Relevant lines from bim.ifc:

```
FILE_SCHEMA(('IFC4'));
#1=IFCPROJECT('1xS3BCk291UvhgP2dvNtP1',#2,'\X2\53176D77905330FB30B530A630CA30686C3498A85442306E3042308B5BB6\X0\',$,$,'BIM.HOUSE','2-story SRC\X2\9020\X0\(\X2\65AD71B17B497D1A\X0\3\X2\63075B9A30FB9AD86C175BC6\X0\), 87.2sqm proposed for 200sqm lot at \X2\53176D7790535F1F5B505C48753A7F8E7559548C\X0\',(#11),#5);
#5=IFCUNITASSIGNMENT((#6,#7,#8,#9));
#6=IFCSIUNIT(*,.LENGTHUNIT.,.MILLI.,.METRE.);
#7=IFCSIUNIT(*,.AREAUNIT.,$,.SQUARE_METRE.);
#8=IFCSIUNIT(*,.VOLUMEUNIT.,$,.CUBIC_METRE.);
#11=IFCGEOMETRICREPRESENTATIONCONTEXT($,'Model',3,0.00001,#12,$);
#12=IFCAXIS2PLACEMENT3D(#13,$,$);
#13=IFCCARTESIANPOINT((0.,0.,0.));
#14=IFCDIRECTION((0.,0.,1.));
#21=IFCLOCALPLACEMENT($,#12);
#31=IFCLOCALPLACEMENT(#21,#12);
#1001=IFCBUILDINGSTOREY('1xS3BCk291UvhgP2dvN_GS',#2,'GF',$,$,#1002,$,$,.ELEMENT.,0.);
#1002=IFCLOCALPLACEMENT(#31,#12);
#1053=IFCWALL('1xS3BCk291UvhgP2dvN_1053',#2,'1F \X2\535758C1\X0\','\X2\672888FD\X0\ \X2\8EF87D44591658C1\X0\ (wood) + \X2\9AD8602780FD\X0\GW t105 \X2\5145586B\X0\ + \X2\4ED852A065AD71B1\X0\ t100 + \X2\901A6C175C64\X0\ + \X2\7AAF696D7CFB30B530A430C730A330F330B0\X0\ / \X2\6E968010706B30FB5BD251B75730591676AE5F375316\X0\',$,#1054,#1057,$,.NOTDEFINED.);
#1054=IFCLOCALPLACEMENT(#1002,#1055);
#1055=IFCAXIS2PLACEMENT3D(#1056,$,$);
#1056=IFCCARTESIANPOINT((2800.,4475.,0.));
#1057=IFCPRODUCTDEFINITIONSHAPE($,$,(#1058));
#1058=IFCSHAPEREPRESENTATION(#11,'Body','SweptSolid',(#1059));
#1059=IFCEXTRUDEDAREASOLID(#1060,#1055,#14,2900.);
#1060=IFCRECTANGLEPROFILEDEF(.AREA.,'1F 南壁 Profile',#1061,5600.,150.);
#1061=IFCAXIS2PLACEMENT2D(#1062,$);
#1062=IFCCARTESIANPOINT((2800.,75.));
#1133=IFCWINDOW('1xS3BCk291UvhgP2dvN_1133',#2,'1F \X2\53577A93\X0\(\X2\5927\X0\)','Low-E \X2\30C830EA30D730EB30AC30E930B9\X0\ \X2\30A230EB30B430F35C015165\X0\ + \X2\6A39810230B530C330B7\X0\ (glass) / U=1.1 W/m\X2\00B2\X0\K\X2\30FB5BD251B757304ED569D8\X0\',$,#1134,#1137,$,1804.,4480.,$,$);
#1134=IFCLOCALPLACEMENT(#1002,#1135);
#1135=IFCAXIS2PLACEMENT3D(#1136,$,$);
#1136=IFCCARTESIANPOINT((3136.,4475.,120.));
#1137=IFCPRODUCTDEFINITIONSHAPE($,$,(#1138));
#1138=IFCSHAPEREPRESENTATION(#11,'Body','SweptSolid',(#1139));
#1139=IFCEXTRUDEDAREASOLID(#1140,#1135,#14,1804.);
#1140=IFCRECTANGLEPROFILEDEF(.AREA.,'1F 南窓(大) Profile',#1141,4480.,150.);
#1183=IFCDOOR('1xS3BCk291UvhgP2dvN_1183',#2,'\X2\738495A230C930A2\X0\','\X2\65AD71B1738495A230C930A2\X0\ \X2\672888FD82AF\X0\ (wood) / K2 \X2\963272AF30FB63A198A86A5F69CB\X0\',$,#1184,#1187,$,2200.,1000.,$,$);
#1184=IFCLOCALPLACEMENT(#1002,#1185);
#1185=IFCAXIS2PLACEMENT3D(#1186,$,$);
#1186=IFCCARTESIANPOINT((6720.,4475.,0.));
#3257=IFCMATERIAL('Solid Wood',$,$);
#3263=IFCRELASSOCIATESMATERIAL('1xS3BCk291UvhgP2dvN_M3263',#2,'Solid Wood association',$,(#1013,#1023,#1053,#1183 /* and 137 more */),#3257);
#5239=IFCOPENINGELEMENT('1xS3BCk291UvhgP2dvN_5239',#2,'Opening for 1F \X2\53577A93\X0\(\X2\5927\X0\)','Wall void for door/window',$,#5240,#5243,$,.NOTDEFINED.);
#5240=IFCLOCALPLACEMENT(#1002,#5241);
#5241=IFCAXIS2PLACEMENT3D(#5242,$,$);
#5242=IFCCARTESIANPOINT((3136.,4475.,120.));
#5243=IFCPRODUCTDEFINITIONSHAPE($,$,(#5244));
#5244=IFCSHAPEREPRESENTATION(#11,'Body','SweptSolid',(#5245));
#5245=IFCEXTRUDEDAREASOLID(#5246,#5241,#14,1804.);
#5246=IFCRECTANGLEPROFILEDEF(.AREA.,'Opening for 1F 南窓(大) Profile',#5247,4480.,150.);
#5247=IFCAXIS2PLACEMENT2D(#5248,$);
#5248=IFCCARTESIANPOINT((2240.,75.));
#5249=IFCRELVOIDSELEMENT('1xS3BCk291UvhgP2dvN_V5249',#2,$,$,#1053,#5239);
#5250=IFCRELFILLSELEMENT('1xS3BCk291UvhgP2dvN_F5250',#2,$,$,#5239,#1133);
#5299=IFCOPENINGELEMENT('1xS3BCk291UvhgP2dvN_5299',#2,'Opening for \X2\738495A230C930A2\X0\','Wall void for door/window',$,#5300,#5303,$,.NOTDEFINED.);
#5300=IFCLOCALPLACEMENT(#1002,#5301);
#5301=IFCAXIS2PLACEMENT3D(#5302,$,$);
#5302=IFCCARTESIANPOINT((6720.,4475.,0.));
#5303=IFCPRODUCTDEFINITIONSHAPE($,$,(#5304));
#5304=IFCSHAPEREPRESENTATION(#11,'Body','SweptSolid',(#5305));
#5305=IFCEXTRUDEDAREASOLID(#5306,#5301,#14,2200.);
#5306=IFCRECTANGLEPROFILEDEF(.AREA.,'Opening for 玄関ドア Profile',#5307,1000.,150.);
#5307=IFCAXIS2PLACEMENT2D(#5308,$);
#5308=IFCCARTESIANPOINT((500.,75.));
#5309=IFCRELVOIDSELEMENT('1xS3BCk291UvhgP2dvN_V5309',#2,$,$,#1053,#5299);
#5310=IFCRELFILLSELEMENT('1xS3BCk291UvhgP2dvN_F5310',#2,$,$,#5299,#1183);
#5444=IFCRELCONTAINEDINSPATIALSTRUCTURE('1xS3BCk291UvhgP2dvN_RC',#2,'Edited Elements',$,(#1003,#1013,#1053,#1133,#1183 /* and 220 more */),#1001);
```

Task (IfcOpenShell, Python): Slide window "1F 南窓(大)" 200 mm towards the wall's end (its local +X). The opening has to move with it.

```python
import ifcopenshell
import ifcopenshell.api.geometry
import ifcopenshell.util.placement
import ifcopenshell.util.unit

model = ifcopenshell.open("bim.ifc")
unit_scale = ifcopenshell.util.unit.calculate_unit_scale(model)

window = model.by_guid("1xS3BCk291UvhgP2dvN_1133")
opening = window.FillsVoids[0].RelatingOpeningElement
wall = opening.VoidsElements[0].RelatingBuildingElement

wall_matrix = ifcopenshell.util.placement.get_local_placement(wall.ObjectPlacement)
shift = wall_matrix[:3, 0] * 0.2 / unit_scale
before = ifcopenshell.util.placement.get_local_placement(window.ObjectPlacement)[:3, 3].copy()

# The window is not placed relative to its opening, so move both.
for product in (opening, window):
    matrix = ifcopenshell.util.placement.get_local_placement(product.ObjectPlacement)
    matrix[:3, 3] += shift
    ifcopenshell.api.geometry.edit_object_placement(model, product=product, matrix=matrix, is_si=False)

after = ifcopenshell.util.placement.get_local_placement(window.ObjectPlacement)[:3, 3]
print("window moved by", (after - before).round(3) + 0.0)

model.write("bim_rev.ifc")
```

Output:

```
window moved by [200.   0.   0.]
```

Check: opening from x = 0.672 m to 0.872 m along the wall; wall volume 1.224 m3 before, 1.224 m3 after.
